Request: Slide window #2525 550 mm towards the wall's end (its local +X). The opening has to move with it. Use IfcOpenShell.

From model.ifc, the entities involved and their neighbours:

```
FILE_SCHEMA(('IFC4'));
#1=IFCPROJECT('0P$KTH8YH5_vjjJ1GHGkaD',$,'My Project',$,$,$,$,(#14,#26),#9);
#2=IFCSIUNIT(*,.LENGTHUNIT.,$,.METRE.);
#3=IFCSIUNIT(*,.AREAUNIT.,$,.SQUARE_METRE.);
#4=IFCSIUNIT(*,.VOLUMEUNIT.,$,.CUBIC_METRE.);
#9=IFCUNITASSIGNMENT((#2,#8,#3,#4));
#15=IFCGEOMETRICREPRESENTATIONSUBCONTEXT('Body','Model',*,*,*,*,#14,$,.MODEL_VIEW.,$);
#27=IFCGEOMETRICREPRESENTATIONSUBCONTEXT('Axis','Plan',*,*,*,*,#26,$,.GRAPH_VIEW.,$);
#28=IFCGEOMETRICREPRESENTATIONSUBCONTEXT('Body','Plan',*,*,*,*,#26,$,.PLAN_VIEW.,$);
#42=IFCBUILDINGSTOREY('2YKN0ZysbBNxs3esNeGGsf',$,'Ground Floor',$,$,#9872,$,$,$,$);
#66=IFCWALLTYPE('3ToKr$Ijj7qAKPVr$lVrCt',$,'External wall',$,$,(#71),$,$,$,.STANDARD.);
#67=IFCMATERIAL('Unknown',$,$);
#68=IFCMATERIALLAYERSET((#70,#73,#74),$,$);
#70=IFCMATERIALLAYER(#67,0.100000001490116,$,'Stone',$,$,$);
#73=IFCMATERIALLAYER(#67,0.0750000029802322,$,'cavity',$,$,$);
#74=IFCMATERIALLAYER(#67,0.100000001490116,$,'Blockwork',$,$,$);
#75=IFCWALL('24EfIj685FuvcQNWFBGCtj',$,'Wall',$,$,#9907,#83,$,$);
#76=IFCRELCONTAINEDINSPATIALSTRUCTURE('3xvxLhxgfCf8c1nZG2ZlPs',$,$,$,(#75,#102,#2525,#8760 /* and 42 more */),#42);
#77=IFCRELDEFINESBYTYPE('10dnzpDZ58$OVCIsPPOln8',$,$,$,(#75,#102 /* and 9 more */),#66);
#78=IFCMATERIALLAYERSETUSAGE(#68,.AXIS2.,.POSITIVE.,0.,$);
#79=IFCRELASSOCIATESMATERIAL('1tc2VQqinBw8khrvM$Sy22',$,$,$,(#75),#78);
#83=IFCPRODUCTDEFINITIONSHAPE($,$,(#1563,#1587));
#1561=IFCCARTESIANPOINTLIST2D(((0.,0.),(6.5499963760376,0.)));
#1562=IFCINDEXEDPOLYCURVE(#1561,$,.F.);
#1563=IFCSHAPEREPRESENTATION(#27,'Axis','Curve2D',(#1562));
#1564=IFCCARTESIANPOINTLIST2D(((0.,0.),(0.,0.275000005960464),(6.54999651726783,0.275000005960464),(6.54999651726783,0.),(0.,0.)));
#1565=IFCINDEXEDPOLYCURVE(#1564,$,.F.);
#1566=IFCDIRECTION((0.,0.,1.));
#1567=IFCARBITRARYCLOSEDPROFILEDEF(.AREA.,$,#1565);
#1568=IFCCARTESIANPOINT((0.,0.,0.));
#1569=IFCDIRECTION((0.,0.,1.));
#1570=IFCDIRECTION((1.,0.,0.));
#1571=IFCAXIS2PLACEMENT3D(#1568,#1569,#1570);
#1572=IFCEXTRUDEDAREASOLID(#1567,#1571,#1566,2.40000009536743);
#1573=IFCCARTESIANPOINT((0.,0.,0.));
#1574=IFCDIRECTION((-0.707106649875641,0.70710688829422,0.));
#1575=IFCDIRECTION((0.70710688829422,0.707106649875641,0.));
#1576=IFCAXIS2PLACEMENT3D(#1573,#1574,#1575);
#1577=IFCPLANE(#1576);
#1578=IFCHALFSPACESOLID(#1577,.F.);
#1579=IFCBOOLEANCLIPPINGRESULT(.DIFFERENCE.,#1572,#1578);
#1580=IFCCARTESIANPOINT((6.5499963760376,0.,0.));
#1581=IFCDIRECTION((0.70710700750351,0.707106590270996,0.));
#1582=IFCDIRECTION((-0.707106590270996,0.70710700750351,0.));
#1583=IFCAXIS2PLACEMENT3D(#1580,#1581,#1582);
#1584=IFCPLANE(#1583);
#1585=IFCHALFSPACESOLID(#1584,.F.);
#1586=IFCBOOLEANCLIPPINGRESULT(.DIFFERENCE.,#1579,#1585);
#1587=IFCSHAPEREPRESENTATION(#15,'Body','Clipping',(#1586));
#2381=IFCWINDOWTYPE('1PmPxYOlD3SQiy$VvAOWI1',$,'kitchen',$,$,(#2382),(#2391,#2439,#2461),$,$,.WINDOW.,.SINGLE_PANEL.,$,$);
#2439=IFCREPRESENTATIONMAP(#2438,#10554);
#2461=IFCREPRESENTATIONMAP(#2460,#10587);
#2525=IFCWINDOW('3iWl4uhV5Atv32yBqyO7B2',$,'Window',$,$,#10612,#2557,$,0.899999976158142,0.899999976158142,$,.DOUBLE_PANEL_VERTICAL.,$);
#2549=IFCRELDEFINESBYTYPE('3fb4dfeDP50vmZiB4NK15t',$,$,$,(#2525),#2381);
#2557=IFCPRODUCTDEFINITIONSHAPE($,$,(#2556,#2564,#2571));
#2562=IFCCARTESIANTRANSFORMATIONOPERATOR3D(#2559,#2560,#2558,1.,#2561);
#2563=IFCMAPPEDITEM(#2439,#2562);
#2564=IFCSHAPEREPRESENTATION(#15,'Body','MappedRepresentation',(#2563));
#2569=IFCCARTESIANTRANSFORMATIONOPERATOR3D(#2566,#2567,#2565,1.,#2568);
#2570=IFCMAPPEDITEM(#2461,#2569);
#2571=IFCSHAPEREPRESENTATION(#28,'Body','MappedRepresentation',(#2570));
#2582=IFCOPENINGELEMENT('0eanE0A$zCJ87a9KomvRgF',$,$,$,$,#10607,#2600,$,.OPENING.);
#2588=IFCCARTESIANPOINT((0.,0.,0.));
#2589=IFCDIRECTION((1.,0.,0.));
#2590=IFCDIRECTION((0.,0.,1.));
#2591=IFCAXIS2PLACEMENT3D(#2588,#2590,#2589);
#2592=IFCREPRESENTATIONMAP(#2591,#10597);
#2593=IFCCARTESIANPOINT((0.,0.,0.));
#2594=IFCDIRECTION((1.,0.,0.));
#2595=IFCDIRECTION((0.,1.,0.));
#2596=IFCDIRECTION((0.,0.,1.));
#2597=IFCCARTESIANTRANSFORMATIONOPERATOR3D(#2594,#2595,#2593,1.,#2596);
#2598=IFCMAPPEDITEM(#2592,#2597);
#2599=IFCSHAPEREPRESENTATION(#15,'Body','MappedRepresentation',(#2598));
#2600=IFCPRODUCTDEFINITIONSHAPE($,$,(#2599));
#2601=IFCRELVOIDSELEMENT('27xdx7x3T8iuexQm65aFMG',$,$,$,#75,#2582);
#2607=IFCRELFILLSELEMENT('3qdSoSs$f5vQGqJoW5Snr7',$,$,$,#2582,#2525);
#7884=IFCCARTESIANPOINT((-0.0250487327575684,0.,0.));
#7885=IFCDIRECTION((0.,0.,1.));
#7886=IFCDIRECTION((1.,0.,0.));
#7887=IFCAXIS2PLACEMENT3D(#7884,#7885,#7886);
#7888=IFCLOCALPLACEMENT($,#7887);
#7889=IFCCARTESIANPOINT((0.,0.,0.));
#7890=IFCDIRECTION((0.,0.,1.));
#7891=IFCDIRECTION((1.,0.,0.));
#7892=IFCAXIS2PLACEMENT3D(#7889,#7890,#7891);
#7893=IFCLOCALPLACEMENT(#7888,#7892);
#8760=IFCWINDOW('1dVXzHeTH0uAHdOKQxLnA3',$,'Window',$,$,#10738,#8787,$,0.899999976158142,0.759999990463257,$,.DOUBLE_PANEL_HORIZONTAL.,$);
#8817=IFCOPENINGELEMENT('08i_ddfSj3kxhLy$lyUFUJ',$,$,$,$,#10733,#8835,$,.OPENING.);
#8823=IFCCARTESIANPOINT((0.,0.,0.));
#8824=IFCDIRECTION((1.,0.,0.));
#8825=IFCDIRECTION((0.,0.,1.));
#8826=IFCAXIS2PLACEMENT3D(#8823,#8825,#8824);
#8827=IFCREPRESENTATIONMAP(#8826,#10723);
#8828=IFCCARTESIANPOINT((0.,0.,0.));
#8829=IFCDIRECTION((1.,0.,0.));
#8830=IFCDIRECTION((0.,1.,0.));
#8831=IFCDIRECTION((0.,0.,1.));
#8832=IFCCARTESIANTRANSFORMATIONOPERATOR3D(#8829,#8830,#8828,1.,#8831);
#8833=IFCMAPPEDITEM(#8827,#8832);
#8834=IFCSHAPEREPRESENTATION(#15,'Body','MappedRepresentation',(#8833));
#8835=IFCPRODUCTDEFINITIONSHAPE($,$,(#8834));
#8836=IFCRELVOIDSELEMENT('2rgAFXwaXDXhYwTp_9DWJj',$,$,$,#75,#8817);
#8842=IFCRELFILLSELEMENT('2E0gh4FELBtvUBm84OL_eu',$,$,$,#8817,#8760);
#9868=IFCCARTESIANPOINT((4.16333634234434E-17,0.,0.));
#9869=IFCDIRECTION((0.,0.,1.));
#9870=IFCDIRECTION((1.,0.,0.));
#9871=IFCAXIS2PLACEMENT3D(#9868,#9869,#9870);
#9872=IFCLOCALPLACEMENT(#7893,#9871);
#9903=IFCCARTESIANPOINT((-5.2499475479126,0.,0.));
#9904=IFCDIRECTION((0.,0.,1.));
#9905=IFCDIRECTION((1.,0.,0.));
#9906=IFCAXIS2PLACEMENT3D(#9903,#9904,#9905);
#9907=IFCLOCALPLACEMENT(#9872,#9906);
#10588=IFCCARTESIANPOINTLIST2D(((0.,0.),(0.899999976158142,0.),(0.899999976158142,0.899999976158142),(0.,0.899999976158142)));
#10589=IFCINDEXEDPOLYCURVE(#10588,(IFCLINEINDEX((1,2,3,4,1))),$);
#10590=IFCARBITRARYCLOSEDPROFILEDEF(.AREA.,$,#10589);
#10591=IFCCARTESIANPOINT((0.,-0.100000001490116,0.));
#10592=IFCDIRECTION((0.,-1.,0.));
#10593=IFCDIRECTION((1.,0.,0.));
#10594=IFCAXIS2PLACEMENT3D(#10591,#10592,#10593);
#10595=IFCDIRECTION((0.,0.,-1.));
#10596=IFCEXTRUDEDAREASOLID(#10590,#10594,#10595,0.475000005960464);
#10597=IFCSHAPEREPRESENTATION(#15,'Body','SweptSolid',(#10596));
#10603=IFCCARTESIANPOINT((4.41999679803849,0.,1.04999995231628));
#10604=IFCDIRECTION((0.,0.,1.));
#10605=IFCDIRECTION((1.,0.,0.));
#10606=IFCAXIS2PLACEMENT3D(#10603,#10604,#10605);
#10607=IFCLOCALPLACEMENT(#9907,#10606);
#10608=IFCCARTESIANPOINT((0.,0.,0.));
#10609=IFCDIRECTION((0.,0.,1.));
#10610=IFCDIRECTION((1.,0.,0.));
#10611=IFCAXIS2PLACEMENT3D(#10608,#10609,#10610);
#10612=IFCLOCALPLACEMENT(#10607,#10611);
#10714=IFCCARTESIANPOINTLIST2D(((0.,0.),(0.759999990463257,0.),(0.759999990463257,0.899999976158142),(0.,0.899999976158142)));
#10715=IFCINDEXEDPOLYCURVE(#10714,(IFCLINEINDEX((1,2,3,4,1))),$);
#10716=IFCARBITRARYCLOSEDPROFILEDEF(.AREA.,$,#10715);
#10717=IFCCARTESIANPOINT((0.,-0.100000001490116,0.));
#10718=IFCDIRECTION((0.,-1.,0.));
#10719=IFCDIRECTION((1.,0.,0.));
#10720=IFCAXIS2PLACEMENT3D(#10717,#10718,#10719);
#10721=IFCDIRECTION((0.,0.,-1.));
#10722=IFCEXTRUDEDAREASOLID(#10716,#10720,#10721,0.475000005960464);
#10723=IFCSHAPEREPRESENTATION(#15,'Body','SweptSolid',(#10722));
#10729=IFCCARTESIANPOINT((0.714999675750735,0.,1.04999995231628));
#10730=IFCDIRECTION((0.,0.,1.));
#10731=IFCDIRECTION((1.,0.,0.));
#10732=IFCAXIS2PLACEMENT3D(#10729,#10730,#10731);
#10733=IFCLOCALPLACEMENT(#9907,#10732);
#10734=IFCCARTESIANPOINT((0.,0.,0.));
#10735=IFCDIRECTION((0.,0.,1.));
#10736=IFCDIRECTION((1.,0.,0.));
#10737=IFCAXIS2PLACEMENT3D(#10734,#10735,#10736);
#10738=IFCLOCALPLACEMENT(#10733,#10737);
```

```python
import ifcopenshell
import ifcopenshell.api.geometry
import ifcopenshell.util.placement

model = ifcopenshell.open("model.ifc")

window = model.by_guid("3iWl4uhV5Atv32yBqyO7B2")
opening = window.FillsVoids[0].RelatingOpeningElement
wall = opening.VoidsElements[0].RelatingBuildingElement

wall_matrix = ifcopenshell.util.placement.get_local_placement(wall.ObjectPlacement)
shift = wall_matrix[:3, 0] * 0.55
before = ifcopenshell.util.placement.get_local_placement(window.ObjectPlacement)[:3, 3].copy()

# The window is placed relative to its opening, so it follows when the opening moves.
matrix = ifcopenshell.util.placement.get_local_placement(opening.ObjectPlacement)
matrix[:3, 3] += shift
ifcopenshell.api.geometry.edit_object_placement(
    model, product=opening, matrix=matrix, is_si=False, should_transform_children=True
)

after = ifcopenshell.util.placement.get_local_placement(window.ObjectPlacement)[:3, 3]
print("window moved by", (after - before).round(3) + 0.0)

model.write("model_updated.ifc")
```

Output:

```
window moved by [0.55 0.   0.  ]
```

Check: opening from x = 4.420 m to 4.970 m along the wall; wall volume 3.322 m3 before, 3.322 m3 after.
